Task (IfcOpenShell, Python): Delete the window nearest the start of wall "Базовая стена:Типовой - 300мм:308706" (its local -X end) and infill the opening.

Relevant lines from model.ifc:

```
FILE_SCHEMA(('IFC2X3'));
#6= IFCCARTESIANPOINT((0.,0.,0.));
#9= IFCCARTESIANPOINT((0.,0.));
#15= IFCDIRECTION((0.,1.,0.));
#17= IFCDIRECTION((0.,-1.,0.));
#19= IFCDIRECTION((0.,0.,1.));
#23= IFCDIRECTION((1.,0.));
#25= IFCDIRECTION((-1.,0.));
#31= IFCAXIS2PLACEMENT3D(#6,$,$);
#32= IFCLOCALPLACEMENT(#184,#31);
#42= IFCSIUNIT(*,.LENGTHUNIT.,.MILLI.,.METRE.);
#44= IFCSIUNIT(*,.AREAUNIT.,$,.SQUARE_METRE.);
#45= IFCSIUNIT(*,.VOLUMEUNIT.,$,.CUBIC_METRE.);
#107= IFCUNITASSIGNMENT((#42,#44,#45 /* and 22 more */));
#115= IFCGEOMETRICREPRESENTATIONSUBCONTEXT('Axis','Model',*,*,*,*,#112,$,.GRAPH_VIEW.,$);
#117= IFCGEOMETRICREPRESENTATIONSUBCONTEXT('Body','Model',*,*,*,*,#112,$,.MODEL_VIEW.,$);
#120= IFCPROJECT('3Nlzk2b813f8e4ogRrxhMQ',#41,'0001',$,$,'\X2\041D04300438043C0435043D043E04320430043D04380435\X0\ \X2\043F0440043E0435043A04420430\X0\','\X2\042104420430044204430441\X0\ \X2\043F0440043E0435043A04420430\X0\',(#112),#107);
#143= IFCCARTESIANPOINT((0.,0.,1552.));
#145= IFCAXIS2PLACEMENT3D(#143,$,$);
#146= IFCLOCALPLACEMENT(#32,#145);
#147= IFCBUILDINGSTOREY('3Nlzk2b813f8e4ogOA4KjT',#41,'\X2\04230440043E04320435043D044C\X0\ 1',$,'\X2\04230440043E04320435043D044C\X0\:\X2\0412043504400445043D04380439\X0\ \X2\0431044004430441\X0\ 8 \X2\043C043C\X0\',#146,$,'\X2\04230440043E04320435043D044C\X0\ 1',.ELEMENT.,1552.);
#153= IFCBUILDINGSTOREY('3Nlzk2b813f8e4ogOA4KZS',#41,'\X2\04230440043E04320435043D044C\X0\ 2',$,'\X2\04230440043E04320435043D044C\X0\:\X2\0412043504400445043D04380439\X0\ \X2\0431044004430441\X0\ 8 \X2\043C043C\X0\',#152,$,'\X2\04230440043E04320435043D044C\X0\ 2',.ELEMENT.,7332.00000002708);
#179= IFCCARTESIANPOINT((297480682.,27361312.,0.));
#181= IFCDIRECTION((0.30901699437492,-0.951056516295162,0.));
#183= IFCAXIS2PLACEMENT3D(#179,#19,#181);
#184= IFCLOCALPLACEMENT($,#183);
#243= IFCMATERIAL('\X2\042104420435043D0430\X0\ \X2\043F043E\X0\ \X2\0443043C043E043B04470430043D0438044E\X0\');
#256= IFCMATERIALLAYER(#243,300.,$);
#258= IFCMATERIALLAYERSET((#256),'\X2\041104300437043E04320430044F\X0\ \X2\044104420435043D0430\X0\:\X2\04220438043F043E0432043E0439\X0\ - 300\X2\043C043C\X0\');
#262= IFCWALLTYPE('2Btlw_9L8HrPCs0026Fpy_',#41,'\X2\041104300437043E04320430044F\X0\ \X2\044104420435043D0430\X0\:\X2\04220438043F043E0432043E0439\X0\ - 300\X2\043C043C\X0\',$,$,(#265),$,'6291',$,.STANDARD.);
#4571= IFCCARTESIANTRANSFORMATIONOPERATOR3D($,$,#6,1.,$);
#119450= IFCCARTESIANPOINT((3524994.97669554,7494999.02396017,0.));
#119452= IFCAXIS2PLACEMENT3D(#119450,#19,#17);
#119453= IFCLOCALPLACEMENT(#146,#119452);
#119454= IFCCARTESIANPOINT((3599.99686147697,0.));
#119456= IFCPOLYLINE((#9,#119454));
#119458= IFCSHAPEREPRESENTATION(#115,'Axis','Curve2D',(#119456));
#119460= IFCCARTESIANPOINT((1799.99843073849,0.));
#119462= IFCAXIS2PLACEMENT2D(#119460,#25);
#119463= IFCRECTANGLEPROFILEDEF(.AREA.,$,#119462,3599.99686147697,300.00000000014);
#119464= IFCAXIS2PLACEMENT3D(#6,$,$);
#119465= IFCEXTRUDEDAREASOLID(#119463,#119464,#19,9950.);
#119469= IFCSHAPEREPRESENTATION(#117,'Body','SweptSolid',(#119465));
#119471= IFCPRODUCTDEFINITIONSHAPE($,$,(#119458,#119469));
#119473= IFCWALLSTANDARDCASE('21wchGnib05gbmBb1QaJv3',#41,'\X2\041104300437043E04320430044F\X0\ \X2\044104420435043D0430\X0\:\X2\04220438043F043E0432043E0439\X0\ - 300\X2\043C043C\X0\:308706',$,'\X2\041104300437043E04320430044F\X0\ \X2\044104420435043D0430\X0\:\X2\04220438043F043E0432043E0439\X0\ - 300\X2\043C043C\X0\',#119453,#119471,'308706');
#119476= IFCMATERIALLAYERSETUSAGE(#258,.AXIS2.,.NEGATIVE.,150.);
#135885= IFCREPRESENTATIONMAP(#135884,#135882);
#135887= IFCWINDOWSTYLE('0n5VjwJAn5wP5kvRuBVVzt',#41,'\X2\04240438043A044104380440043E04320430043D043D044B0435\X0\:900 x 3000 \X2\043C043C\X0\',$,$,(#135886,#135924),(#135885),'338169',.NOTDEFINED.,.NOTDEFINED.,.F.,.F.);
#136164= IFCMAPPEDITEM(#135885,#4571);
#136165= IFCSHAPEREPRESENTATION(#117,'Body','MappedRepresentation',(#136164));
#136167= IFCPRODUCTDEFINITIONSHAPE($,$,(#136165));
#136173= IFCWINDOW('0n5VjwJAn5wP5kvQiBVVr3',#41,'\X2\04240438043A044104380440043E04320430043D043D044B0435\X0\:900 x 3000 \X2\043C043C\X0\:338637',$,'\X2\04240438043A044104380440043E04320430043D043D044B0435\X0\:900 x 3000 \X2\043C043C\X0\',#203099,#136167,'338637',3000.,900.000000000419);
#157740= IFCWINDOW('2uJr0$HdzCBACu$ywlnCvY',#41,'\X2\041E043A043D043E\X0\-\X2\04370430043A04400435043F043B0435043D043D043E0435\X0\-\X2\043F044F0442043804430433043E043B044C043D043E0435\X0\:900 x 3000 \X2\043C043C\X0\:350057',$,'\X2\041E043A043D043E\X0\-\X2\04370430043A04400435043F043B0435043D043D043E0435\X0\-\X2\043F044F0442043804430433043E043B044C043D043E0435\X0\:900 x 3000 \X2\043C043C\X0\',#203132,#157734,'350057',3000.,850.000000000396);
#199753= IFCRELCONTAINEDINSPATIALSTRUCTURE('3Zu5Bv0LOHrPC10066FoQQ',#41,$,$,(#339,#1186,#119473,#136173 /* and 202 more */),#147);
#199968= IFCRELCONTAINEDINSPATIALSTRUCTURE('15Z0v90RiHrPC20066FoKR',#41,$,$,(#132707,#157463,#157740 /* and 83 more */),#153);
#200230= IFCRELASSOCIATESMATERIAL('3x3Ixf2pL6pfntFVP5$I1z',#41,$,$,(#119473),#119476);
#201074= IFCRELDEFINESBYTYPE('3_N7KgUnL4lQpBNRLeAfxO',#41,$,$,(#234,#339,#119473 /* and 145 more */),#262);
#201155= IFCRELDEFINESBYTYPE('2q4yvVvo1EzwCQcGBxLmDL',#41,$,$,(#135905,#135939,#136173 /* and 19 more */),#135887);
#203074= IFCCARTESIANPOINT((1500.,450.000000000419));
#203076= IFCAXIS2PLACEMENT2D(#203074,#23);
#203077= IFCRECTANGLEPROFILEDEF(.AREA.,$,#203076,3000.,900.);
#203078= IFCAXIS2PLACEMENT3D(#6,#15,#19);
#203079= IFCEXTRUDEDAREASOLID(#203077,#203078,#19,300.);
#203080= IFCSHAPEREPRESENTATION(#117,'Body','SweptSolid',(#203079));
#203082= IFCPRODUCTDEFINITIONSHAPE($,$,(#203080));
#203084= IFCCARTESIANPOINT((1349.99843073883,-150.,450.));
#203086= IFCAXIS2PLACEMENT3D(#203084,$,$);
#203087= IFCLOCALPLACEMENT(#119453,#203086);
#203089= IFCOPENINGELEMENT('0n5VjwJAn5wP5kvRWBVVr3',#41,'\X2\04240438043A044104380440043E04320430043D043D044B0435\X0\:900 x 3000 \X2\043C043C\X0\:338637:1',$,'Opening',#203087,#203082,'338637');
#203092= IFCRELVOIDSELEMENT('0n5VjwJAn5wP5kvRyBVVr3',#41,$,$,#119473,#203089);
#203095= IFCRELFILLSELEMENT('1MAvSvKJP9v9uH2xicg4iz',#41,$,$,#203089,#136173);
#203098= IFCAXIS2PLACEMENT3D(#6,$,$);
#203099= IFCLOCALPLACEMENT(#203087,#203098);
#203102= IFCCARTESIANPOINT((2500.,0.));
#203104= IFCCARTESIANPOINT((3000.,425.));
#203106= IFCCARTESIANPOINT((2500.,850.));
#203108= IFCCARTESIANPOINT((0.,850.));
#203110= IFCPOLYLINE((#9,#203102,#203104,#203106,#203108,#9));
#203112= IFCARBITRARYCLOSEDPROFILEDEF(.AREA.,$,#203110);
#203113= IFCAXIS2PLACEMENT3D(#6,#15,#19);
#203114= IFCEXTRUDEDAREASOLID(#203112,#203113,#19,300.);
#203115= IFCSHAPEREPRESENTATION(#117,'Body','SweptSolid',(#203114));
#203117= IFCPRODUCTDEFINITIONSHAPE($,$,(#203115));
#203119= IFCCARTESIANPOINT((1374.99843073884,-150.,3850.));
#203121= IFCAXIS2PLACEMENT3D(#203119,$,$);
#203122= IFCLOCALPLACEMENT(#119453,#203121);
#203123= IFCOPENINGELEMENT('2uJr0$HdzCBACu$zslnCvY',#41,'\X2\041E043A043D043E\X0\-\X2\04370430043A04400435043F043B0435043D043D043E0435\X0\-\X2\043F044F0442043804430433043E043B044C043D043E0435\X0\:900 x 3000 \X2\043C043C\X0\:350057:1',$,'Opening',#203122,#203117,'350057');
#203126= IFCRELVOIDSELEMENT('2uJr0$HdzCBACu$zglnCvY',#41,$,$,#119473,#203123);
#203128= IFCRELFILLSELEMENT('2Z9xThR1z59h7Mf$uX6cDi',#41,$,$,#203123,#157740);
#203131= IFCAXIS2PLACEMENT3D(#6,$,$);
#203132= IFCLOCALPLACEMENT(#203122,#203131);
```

```python
import ifcopenshell
import ifcopenshell.api.feature
import ifcopenshell.api.root
import ifcopenshell.geom
import ifcopenshell.util.shape

model = ifcopenshell.open("model.ifc")
settings = ifcopenshell.geom.settings()


def volume(element):
    """Net volume in cubic metres, openings subtracted."""
    shape = ifcopenshell.geom.create_shape(settings, element)
    return ifcopenshell.util.shape.get_volume(shape.geometry)


window = model.by_guid("0n5VjwJAn5wP5kvQiBVVr3")
opening = window.FillsVoids[0].RelatingOpeningElement
wall = opening.VoidsElements[0].RelatingBuildingElement
before = volume(wall)

ifcopenshell.api.root.remove_product(model, product=window)
ifcopenshell.api.feature.remove_feature(model, feature=opening)

after = volume(wall)

print(f"wall volume {before:.3f} -> {after:.3f} m3")

model.write("model_v2.ifc")
```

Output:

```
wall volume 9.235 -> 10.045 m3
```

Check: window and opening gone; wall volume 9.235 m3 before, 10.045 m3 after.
